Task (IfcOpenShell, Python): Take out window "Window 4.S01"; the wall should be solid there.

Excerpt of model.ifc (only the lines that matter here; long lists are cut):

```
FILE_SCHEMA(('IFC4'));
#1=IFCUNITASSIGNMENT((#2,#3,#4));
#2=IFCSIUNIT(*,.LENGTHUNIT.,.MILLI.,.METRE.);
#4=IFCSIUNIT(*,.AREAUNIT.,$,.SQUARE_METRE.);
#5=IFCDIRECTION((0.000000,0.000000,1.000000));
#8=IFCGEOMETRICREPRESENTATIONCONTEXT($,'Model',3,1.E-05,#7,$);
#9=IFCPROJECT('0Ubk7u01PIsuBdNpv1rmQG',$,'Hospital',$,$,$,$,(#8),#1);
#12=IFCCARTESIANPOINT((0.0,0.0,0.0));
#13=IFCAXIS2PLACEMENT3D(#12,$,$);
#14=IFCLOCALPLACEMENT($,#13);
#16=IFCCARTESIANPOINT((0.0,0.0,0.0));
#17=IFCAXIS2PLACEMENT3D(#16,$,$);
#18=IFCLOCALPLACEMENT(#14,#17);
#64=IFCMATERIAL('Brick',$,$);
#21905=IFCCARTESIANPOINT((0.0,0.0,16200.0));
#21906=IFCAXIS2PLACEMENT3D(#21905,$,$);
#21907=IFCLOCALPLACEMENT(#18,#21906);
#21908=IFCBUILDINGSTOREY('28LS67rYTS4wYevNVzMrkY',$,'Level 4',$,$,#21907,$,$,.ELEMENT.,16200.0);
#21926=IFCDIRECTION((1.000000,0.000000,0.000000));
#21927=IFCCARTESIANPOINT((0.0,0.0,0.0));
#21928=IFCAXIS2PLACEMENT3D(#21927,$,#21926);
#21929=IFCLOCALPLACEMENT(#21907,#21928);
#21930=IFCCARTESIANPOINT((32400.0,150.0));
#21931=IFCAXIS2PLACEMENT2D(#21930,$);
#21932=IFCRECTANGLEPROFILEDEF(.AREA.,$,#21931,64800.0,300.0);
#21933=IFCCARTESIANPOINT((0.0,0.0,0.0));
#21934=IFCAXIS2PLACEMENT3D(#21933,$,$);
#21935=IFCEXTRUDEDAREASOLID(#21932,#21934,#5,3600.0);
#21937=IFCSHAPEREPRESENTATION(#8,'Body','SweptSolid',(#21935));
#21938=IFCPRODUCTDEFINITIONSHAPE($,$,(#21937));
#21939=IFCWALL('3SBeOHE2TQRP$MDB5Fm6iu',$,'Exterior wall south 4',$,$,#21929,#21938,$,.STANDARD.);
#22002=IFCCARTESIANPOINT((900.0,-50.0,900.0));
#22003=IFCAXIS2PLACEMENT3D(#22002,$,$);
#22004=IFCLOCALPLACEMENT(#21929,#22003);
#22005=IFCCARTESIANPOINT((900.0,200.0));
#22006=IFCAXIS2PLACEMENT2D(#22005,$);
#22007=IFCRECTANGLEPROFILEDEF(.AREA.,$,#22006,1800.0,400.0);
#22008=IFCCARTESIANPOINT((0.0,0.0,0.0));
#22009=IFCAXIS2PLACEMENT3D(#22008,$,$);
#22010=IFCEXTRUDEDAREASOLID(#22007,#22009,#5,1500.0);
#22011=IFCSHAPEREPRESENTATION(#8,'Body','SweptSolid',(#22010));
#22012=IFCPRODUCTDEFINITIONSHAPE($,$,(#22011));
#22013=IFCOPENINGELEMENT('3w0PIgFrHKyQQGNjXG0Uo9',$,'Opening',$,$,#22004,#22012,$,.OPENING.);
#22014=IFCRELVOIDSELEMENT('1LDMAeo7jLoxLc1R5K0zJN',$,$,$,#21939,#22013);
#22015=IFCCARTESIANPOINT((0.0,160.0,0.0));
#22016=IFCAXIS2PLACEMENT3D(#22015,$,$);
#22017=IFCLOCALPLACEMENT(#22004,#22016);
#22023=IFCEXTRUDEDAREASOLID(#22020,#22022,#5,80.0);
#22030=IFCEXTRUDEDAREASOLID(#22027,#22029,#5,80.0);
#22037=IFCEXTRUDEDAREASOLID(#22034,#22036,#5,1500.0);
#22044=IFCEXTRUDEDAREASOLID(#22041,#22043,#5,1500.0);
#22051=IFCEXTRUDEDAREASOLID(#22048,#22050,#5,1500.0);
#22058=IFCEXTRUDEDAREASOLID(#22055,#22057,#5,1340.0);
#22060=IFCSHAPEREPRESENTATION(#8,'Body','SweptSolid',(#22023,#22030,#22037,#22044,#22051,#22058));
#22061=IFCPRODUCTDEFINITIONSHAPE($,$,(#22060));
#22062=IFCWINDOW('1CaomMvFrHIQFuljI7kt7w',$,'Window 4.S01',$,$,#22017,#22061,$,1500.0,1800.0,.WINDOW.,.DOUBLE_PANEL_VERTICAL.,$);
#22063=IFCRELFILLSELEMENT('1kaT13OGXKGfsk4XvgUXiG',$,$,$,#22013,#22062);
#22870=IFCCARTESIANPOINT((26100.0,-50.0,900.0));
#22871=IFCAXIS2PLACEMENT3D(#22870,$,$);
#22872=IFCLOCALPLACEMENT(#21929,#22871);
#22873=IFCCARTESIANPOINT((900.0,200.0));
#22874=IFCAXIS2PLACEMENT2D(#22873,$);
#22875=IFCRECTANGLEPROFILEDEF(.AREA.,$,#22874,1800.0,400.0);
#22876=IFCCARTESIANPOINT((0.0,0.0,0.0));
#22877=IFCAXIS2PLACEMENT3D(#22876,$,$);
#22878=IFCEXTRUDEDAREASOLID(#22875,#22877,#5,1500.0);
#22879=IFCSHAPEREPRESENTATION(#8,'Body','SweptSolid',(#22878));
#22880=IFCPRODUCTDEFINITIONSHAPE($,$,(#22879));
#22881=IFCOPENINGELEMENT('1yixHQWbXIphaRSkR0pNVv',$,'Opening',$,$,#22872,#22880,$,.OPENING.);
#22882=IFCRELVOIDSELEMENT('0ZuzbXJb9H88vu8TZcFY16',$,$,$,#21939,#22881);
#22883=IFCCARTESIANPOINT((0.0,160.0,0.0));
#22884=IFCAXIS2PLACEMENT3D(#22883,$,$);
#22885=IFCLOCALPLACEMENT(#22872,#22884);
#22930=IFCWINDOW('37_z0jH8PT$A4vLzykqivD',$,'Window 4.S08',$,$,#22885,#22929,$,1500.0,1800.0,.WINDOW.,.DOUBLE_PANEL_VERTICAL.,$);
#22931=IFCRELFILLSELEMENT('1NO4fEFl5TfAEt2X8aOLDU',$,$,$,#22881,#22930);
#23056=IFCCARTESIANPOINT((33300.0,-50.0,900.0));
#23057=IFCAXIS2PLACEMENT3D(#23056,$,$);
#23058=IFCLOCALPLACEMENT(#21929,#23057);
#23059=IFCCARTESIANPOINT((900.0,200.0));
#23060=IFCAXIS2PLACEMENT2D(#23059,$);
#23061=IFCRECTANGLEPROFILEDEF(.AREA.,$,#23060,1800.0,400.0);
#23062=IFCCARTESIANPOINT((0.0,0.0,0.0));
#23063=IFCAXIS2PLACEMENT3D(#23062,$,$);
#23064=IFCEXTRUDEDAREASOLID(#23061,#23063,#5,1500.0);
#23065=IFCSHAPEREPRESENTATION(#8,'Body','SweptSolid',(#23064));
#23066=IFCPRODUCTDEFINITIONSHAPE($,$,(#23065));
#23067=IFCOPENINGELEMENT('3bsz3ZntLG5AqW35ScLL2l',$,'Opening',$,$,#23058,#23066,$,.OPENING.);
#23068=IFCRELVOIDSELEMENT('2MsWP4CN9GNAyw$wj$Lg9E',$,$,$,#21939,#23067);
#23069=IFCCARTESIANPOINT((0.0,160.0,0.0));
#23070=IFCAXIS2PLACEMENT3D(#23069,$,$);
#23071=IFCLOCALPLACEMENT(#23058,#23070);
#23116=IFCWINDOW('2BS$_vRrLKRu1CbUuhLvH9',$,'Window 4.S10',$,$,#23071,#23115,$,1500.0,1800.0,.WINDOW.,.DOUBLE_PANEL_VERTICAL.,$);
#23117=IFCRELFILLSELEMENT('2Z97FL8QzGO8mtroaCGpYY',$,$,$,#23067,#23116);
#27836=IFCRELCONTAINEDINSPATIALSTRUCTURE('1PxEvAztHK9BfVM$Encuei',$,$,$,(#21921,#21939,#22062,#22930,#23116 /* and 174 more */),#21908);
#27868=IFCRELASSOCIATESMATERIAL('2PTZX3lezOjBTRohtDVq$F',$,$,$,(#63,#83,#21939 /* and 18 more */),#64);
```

```python
import ifcopenshell
import ifcopenshell.api.feature
import ifcopenshell.api.root
import ifcopenshell.geom
import ifcopenshell.util.shape

model = ifcopenshell.open("model.ifc")
settings = ifcopenshell.geom.settings()


def volume(element):
    """Net volume in cubic metres, openings subtracted."""
    shape = ifcopenshell.geom.create_shape(settings, element)
    return ifcopenshell.util.shape.get_volume(shape.geometry)


window = model.by_guid("1CaomMvFrHIQFuljI7kt7w")
opening = window.FillsVoids[0].RelatingOpeningElement
wall = opening.VoidsElements[0].RelatingBuildingElement
before = volume(wall)

ifcopenshell.api.root.remove_product(model, product=window)
ifcopenshell.api.feature.remove_feature(model, feature=opening)

after = volume(wall)

print(f"wall volume {before:.3f} -> {after:.3f} m3")

model.write("model_edited.ifc")
```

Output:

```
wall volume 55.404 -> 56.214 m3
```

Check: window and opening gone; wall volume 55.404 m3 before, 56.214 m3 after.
